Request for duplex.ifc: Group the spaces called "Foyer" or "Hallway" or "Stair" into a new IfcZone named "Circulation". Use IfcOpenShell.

First a look at what the model holds.

```python
import ifcopenshell

model = ifcopenshell.open("duplex.ifc")
print(model.schema)
seen = {}
for space in model.by_type("IfcSpace"):
    seen[space.LongName] = seen.get(space.LongName, 0) + 1
for name, count in sorted(seen.items(), key=str):
    print(count, "x", name)
print("zones:", [z.Name for z in model.by_type("IfcZone")][:20])
```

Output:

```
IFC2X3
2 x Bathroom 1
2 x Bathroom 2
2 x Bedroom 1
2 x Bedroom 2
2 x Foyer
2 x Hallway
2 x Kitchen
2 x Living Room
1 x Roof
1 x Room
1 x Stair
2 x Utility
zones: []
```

```python
import ifcopenshell
import ifcopenshell.api.group
import ifcopenshell.api.root

model = ifcopenshell.open("duplex.ifc")

names = {"Foyer", "Hallway", "Stair"}
spaces = [s for s in model.by_type("IfcSpace") if s.LongName in names]

zone = ifcopenshell.api.root.create_entity(model, ifc_class="IfcZone", name="Circulation")
ifcopenshell.api.group.assign_group(model, products=spaces, group=zone)
print(len(spaces), "spaces in", zone.Name)

model.write("duplex_rev.ifc")
```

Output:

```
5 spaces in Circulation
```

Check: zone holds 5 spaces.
